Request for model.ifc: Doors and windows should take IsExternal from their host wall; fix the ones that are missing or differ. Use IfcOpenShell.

First a look at what the model holds.

```python
import ifcopenshell
import ifcopenshell.util.element

model = ifcopenshell.open("model.ifc")
print(model.schema)
seen = {}
for e in model.by_type("IfcDoor") + model.by_type("IfcWindow"):
    if not e.FillsVoids:
        continue
    host = e.FillsVoids[0].RelatingOpeningElement.VoidsElements[0].RelatingBuildingElement
    own = ifcopenshell.util.element.get_pset(e, f"Pset_{e.is_a()[3:].removesuffix('StandardCase')}Common", "IsExternal")
    wall = ifcopenshell.util.element.get_pset(host, "Pset_WallCommon", "IsExternal")
    seen[e.is_a(), own, wall] = seen.get((e.is_a(), own, wall), 0) + 1
for (cls, own, wall), count in sorted(seen.items(), key=str):
    print(count, cls, "IsExternal:", own, "| host wall:", wall)
```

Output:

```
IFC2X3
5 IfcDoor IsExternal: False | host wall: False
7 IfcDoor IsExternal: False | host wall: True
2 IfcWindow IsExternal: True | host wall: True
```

```python
import ifcopenshell
import ifcopenshell.api.pset
import ifcopenshell.util.element

model = ifcopenshell.open("model.ifc")

count = 0
for ifc_class, pset_name in (("IfcDoor", "Pset_DoorCommon"), ("IfcWindow", "Pset_WindowCommon")):
    for e in model.by_type(ifc_class):
        if not e.FillsVoids:
            continue
        host = e.FillsVoids[0].RelatingOpeningElement.VoidsElements[0].RelatingBuildingElement
        external = ifcopenshell.util.element.get_pset(host, "Pset_WallCommon", "IsExternal")
        if external is None or ifcopenshell.util.element.get_pset(e, pset_name, "IsExternal") == external:
            continue
        pset = ifcopenshell.api.pset.add_pset(model, product=e, name=pset_name)
        ifcopenshell.api.pset.edit_pset(model, pset=pset, properties={"IsExternal": external})
        count += 1

print(count, "updated")

model.write("model-out.ifc")
```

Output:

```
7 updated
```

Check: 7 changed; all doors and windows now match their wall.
